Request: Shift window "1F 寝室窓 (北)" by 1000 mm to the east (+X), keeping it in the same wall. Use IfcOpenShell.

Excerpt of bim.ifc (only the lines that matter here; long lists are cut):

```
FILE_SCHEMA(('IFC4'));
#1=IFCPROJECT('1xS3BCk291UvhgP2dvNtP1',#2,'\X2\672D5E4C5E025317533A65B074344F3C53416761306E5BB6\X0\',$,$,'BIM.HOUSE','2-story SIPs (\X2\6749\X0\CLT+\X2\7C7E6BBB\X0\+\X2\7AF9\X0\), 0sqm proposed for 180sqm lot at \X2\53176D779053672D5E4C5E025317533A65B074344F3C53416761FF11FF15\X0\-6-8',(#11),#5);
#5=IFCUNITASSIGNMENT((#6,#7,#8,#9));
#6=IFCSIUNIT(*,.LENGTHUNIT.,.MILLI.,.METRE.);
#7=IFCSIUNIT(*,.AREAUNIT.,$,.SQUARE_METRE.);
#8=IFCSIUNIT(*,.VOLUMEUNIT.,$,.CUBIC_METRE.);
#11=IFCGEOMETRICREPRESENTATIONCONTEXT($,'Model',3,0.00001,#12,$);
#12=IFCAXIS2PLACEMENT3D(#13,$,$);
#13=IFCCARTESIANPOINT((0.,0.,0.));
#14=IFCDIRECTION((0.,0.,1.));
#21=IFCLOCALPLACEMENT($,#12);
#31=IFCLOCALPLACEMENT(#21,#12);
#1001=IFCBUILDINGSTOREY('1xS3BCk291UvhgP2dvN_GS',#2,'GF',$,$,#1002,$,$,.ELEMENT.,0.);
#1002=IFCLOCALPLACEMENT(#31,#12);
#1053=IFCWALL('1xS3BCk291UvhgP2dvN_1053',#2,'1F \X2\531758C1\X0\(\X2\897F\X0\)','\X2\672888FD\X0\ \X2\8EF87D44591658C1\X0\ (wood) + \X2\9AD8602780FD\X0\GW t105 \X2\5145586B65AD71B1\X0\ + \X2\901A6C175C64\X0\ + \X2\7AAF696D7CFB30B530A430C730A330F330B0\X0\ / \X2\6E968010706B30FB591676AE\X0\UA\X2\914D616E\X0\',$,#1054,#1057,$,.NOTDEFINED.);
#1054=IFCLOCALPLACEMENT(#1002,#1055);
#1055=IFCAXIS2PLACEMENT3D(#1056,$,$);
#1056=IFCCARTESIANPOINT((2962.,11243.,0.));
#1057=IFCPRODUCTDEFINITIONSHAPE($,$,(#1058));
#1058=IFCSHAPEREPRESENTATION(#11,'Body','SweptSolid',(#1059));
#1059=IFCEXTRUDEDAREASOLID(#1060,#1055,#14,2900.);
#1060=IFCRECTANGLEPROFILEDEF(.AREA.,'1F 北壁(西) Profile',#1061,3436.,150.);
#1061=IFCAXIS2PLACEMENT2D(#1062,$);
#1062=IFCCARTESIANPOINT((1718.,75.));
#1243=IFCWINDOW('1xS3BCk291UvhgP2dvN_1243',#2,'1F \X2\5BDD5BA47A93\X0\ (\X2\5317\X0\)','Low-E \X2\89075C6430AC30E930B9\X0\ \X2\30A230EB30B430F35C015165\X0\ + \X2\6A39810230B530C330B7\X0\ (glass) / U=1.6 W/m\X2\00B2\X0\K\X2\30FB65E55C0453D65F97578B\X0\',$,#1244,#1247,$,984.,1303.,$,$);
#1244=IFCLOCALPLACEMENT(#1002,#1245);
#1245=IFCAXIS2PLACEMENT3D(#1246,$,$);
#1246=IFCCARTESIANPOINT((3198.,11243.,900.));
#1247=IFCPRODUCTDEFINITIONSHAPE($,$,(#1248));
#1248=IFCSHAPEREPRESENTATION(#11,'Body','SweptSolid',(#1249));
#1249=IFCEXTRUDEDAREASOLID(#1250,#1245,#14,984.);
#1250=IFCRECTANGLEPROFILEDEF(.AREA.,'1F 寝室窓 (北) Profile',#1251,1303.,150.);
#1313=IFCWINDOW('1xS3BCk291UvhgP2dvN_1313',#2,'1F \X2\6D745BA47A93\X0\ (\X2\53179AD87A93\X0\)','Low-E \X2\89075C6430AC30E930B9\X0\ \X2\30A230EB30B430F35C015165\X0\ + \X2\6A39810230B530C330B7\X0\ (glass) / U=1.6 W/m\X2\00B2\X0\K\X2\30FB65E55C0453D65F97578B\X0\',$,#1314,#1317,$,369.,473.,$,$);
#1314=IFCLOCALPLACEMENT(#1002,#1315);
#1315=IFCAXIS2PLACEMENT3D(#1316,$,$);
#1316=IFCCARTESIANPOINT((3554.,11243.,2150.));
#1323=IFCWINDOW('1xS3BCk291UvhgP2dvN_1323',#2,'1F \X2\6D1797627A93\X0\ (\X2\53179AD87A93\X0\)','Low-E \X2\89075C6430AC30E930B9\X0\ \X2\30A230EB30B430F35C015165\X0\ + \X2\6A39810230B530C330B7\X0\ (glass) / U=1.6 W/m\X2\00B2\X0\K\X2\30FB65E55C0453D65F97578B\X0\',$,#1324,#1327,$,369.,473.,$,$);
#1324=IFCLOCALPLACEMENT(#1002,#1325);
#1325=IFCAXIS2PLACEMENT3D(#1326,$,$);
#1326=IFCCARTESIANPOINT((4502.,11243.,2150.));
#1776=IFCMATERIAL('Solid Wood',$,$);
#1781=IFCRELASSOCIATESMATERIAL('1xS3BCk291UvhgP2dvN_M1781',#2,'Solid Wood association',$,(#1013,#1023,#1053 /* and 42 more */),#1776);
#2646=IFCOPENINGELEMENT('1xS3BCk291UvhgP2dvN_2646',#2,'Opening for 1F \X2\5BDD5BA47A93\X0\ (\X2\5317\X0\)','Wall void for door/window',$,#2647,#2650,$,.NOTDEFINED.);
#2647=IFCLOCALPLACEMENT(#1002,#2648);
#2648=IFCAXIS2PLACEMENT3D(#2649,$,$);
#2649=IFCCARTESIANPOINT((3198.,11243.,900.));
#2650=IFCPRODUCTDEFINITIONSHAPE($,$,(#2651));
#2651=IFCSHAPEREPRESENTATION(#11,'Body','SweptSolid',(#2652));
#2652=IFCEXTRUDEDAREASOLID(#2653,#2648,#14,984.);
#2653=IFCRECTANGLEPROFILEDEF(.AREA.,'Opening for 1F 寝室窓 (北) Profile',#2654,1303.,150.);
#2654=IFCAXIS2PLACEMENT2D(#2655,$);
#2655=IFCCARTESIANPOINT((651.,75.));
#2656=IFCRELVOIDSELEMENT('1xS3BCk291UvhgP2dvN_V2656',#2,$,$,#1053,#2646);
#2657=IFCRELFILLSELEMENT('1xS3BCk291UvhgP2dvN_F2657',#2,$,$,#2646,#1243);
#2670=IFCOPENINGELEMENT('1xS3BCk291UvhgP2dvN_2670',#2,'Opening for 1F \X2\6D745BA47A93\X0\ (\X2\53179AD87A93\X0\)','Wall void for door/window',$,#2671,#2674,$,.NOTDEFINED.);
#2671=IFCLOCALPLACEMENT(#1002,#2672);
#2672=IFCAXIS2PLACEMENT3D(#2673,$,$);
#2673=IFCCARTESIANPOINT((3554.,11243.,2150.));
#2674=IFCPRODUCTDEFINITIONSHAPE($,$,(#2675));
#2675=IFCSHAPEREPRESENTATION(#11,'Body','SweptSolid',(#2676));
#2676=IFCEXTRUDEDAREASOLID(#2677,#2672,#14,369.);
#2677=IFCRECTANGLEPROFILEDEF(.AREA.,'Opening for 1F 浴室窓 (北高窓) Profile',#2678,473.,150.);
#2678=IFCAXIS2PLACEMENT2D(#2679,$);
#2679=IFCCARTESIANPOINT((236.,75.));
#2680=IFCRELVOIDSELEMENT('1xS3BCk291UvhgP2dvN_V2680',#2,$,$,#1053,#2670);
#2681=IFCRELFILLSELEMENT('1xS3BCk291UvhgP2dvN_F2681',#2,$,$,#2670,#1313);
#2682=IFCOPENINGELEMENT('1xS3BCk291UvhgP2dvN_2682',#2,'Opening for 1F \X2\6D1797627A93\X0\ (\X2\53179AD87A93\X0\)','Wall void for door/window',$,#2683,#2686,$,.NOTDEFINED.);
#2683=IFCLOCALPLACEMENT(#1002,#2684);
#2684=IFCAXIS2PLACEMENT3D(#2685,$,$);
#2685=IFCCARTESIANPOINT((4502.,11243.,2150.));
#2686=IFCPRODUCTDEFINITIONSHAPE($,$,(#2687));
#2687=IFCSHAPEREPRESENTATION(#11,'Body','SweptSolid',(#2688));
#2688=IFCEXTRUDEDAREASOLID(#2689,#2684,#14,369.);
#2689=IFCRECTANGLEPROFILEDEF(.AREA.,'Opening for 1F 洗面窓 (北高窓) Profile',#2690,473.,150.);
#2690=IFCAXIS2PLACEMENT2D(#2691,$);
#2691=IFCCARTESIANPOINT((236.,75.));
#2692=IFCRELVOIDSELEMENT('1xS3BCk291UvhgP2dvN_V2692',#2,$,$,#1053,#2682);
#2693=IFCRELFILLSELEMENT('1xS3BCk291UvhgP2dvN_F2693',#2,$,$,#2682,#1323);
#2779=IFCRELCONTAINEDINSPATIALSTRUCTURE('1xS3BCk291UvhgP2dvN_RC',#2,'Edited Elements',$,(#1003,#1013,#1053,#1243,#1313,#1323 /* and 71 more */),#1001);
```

```python
import ifcopenshell
import ifcopenshell.api.geometry
import ifcopenshell.util.placement
import ifcopenshell.util.unit

model = ifcopenshell.open("bim.ifc")
unit_scale = ifcopenshell.util.unit.calculate_unit_scale(model)

window = model.by_id(1243)
opening = window.FillsVoids[0].RelatingOpeningElement
wall = opening.VoidsElements[0].RelatingBuildingElement

wall_matrix = ifcopenshell.util.placement.get_local_placement(wall.ObjectPlacement)
shift = wall_matrix[:3, 0] * 1 / unit_scale
before = ifcopenshell.util.placement.get_local_placement(window.ObjectPlacement)[:3, 3].copy()

# The window is not placed relative to its opening, so move both.
for product in (opening, window):
    matrix = ifcopenshell.util.placement.get_local_placement(product.ObjectPlacement)
    matrix[:3, 3] += shift
    ifcopenshell.api.geometry.edit_object_placement(model, product=product, matrix=matrix, is_si=False)

after = ifcopenshell.util.placement.get_local_placement(window.ObjectPlacement)[:3, 3]
print("window moved by", (after - before).round(3) + 0.0)

model.write("bim_updated.ifc")
```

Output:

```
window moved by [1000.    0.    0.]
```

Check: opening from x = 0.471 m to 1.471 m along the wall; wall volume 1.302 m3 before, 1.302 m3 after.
